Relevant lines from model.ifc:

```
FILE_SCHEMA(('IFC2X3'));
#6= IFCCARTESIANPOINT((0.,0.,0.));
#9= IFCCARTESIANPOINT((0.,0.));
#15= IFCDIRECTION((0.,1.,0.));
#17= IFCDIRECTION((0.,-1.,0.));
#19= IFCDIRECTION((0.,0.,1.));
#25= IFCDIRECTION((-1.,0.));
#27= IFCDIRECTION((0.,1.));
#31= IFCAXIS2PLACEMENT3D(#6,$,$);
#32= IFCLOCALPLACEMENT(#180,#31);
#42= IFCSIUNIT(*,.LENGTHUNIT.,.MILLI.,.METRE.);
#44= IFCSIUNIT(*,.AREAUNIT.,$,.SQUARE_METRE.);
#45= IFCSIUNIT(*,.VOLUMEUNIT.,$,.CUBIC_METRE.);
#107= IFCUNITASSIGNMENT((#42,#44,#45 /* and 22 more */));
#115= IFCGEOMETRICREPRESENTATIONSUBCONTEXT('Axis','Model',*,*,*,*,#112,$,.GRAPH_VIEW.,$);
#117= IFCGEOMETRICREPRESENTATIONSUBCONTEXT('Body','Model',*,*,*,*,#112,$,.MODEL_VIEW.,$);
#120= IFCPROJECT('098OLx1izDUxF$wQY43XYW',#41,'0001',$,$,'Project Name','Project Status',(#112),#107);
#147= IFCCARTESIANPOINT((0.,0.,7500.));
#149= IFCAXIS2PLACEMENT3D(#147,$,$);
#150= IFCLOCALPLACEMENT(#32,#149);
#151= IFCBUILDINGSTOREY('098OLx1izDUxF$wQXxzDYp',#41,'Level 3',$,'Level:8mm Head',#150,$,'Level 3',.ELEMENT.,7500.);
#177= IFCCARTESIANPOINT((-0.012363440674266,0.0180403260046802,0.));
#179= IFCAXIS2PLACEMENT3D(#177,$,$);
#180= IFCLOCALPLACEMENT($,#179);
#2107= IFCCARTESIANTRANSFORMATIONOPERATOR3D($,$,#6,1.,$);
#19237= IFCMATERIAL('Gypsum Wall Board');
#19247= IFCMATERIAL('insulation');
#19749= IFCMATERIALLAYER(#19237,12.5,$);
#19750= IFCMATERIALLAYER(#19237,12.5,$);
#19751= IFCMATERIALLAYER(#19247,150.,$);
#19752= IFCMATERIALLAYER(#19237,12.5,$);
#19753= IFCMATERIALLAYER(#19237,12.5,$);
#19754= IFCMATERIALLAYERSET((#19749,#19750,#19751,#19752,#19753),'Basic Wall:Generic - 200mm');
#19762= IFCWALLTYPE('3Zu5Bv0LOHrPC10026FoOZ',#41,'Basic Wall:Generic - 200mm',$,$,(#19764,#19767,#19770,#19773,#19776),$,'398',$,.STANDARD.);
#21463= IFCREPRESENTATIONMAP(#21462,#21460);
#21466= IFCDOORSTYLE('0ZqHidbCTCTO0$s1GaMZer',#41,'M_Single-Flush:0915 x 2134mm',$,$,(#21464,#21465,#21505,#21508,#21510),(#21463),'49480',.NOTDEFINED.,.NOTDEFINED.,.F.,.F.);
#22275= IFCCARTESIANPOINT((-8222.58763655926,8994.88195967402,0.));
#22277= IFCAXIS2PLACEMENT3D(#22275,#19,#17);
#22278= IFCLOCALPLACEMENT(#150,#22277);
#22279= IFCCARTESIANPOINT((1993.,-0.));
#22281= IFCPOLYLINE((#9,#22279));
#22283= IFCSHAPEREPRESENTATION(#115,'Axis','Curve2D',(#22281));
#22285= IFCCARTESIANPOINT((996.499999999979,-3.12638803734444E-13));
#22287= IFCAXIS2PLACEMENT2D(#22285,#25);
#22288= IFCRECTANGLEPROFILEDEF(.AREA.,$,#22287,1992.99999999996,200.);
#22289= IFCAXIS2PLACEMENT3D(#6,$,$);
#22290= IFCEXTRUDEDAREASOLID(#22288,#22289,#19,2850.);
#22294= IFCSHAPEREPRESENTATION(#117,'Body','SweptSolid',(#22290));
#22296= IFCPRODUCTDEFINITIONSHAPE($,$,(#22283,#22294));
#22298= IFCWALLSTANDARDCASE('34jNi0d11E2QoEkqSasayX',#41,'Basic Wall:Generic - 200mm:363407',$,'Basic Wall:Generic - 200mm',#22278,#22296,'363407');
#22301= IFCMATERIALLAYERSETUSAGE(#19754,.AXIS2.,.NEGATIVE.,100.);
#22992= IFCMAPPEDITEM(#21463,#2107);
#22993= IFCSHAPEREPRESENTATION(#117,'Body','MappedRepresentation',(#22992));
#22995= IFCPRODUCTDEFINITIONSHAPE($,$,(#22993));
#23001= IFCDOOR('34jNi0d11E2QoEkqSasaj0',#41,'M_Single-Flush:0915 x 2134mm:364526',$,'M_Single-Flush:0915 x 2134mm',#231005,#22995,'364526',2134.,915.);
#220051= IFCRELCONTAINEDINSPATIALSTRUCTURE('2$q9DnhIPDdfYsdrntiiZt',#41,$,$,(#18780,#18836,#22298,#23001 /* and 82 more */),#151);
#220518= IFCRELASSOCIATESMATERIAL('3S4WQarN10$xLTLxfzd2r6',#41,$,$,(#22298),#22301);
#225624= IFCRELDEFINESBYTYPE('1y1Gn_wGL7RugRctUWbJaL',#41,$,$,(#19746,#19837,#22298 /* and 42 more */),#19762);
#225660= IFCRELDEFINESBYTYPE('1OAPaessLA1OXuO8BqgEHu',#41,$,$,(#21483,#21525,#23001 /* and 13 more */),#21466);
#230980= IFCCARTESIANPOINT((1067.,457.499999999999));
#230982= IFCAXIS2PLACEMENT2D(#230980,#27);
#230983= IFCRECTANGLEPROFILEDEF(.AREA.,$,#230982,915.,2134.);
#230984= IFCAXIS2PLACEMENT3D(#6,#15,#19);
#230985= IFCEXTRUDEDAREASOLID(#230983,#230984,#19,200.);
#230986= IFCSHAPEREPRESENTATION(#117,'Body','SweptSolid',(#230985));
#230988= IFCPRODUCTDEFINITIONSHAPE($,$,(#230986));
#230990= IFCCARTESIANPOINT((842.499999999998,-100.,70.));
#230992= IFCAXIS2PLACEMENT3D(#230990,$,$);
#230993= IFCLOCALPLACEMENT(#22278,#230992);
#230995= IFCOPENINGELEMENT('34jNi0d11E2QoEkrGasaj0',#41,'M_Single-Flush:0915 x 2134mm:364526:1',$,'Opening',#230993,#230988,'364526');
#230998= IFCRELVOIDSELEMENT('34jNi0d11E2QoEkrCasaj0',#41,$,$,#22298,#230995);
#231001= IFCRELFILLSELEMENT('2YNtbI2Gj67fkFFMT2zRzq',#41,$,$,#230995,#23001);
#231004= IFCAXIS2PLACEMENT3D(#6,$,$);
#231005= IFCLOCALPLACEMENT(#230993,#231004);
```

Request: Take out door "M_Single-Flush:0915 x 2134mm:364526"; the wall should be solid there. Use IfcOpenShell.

```python
import ifcopenshell
import ifcopenshell.api.feature
import ifcopenshell.api.root
import ifcopenshell.geom
import ifcopenshell.util.shape

model = ifcopenshell.open("model.ifc")
settings = ifcopenshell.geom.settings()


def volume(element):
    """Net volume in cubic metres, openings subtracted."""
    shape = ifcopenshell.geom.create_shape(settings, element)
    return ifcopenshell.util.shape.get_volume(shape.geometry)


door = model.by_id(23001)
opening = door.FillsVoids[0].RelatingOpeningElement
wall = opening.VoidsElements[0].RelatingBuildingElement
before = volume(wall)

ifcopenshell.api.root.remove_product(model, product=door)
ifcopenshell.api.feature.remove_feature(model, feature=opening)

after = volume(wall)

print(f"wall volume {before:.3f} -> {after:.3f} m3")

model.write("model_v2.ifc")
```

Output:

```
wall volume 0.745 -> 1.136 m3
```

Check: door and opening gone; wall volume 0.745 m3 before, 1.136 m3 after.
